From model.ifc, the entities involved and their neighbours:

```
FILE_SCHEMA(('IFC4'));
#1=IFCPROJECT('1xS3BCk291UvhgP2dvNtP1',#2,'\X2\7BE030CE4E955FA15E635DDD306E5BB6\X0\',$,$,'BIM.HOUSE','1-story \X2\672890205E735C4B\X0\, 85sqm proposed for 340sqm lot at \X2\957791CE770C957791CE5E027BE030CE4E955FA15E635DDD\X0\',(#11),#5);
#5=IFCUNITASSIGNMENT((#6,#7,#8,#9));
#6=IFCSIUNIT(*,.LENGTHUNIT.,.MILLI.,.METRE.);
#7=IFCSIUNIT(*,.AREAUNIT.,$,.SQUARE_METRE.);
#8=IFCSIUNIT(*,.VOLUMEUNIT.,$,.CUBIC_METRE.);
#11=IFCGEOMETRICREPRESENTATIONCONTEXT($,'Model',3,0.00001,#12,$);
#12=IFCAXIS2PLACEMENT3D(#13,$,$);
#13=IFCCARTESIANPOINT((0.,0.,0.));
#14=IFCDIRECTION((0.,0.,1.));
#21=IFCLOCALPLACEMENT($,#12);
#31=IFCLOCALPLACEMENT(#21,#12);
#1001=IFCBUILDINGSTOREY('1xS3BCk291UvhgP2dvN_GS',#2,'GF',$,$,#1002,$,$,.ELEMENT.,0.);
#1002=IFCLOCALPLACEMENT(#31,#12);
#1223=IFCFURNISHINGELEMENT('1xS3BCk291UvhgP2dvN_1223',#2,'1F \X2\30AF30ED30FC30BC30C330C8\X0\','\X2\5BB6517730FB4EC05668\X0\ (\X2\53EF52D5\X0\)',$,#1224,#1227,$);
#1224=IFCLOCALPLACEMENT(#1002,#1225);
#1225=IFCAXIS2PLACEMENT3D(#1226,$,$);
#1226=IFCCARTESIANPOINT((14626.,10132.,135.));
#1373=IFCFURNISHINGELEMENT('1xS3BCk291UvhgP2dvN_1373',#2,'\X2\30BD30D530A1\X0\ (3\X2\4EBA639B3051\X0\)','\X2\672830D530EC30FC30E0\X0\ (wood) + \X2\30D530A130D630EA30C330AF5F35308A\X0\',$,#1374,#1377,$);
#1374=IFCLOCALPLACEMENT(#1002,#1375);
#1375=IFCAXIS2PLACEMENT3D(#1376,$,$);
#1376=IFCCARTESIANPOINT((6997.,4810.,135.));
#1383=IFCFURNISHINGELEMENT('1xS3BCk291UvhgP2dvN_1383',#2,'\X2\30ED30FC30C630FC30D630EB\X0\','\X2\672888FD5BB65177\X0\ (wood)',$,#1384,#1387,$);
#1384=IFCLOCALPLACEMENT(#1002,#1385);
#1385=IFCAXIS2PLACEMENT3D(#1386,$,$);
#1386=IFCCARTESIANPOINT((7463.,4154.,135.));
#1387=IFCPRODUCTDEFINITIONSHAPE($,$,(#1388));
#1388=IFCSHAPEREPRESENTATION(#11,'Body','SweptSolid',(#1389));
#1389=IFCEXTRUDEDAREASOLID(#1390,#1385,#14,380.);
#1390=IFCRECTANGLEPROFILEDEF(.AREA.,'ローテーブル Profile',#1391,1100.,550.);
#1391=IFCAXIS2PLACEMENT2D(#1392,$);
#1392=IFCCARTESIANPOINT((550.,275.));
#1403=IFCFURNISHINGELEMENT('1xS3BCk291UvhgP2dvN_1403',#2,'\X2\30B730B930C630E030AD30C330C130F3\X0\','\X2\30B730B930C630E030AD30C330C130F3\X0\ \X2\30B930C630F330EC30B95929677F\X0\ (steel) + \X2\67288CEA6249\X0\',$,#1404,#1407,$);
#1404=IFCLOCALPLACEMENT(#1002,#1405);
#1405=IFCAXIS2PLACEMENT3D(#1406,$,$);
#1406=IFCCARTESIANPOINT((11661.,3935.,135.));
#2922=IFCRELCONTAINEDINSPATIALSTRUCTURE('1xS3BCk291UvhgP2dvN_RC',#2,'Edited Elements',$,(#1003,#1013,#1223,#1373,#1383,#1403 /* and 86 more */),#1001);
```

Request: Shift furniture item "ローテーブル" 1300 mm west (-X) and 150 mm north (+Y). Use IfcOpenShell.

```python
import ifcopenshell
import ifcopenshell.api.geometry
import ifcopenshell.util.placement
import ifcopenshell.util.unit

model = ifcopenshell.open("model.ifc")
unit_scale = ifcopenshell.util.unit.calculate_unit_scale(model)

item = model.by_id(1383)
matrix = ifcopenshell.util.placement.get_local_placement(item.ObjectPlacement)
matrix[0, 3] -= 1.3 / unit_scale
matrix[1, 3] += 0.15 / unit_scale
ifcopenshell.api.geometry.edit_object_placement(model, product=item, matrix=matrix, is_si=False)

print(ifcopenshell.util.placement.get_local_placement(item.ObjectPlacement).round(3) + 0.0)

model.write("model_updated.ifc")
```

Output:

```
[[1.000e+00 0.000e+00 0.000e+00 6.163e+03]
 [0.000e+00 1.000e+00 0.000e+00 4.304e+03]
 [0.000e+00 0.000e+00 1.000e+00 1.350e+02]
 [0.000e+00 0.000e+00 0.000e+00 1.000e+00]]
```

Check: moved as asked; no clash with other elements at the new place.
